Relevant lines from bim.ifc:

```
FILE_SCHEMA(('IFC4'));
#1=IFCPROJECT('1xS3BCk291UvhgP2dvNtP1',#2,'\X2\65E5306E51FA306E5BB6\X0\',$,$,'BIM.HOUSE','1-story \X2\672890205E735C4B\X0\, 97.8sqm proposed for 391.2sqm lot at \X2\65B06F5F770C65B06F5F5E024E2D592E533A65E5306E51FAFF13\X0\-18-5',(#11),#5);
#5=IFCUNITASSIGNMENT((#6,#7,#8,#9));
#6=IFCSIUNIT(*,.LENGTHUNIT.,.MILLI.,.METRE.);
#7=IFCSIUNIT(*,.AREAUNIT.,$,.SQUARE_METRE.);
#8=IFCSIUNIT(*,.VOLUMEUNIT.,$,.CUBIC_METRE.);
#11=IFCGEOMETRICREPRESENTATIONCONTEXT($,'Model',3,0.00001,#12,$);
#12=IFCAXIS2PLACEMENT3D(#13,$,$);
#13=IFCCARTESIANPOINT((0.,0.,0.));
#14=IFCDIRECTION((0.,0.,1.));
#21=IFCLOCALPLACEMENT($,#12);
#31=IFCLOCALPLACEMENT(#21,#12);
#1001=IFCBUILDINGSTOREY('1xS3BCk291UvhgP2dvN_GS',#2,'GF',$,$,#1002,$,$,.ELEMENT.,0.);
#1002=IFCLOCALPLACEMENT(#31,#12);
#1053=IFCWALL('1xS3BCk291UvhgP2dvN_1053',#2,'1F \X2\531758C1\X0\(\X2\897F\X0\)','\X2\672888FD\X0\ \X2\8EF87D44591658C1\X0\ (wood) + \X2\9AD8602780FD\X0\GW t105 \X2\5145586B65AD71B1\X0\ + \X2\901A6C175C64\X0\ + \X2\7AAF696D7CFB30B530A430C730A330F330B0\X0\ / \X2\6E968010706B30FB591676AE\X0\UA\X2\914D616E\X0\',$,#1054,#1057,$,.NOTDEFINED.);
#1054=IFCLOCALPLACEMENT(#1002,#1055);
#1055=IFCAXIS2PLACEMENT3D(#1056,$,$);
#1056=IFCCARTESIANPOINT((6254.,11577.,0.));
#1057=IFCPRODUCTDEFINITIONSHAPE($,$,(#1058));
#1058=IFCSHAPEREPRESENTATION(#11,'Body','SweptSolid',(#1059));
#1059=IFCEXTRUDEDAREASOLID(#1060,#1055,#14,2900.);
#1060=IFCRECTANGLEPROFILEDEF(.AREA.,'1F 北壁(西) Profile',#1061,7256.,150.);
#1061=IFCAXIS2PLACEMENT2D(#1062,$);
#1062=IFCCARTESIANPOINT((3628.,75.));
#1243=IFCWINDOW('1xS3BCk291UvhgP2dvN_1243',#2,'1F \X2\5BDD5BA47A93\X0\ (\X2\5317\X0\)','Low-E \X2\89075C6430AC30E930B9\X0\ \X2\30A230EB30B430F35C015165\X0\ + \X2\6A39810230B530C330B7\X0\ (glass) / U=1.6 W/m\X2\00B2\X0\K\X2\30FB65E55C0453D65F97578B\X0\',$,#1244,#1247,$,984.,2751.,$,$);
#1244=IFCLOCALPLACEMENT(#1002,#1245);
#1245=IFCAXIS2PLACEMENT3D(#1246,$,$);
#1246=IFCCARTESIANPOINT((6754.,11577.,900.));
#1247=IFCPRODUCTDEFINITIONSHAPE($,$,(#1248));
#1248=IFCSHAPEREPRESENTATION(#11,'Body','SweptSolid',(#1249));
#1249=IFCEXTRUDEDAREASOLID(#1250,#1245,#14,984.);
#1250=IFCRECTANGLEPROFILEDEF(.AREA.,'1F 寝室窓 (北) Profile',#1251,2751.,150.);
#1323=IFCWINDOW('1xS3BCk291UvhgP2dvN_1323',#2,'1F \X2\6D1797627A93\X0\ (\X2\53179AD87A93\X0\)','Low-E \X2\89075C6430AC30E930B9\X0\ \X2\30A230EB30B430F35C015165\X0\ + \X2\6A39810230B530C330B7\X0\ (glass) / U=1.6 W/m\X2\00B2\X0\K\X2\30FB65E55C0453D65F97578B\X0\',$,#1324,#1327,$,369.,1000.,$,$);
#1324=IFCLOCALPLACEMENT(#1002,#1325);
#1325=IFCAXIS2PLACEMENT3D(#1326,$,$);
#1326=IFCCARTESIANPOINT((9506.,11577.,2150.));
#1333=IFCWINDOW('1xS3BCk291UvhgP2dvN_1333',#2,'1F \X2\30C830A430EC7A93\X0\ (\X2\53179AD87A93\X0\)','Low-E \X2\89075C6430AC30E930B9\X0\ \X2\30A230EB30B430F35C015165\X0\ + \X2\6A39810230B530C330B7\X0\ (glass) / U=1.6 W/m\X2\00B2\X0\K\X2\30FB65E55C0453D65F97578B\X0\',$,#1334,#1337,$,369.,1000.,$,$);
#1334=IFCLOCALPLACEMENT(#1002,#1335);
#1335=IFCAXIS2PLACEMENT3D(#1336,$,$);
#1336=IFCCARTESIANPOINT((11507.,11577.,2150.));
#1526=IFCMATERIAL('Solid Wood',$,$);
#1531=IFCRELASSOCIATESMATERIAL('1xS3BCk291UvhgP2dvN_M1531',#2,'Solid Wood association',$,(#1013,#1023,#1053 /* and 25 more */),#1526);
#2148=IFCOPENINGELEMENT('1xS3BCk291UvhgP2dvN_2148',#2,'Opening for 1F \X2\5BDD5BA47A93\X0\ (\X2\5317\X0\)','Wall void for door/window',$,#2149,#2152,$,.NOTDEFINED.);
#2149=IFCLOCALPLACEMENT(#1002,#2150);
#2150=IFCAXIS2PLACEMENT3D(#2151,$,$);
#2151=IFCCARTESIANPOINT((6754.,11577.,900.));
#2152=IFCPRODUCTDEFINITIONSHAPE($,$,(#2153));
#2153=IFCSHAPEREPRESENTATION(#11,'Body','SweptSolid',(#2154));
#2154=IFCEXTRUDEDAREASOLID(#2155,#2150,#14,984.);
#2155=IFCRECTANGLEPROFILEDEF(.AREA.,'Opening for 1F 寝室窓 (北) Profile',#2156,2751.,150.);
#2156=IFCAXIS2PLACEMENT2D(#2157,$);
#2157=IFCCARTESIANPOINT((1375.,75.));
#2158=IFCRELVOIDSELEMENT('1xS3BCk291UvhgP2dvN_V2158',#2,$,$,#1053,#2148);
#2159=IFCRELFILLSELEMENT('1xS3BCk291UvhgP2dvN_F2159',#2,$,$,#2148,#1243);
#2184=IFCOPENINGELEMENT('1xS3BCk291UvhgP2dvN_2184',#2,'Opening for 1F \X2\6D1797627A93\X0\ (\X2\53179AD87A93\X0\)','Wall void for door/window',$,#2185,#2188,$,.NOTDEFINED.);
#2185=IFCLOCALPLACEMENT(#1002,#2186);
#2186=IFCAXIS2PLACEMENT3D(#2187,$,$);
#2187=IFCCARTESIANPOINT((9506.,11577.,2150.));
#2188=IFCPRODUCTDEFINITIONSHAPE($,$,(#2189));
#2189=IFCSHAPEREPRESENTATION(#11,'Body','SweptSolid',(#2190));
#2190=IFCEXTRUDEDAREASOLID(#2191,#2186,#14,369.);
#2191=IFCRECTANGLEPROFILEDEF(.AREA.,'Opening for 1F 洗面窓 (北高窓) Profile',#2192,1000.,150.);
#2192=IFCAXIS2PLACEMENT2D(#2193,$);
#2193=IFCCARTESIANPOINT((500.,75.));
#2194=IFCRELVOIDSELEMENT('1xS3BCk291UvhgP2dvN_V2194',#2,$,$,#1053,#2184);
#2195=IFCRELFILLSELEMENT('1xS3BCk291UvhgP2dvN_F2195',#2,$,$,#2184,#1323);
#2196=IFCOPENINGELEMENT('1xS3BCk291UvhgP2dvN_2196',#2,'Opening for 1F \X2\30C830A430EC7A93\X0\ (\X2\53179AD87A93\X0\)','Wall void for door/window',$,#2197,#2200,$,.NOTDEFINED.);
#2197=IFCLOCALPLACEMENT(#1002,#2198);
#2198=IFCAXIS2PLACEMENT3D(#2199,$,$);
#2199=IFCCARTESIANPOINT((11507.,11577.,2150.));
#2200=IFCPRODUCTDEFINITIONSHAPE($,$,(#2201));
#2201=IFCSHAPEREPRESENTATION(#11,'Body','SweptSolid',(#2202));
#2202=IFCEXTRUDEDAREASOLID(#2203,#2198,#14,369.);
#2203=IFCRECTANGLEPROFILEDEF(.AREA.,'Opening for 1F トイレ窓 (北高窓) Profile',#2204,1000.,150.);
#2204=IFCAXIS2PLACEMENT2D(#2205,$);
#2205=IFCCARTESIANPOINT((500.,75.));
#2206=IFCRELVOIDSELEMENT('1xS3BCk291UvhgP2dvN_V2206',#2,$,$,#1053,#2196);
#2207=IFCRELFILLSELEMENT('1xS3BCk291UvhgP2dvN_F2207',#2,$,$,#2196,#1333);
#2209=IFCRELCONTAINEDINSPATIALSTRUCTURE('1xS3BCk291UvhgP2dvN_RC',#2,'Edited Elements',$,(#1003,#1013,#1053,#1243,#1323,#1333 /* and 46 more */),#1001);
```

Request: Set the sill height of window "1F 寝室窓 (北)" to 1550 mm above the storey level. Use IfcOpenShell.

```python
import numpy as np
import ifcopenshell
import ifcopenshell.api.geometry
import ifcopenshell.geom
import ifcopenshell.util.element
import ifcopenshell.util.placement
import ifcopenshell.util.shape
import ifcopenshell.util.unit

model = ifcopenshell.open("bim.ifc")
unit_scale = ifcopenshell.util.unit.calculate_unit_scale(model)

window = model.by_guid("1xS3BCk291UvhgP2dvN_1243")
opening = window.FillsVoids[0].RelatingOpeningElement
storey = ifcopenshell.util.element.get_container(window, ifc_class="IfcBuildingStorey")
level = ifcopenshell.util.placement.get_local_placement(storey.ObjectPlacement)[2, 3]

# The opening's origin need not be at the sill, so measure its lowest point.
shape = ifcopenshell.geom.create_shape(ifcopenshell.geom.settings(), opening)
bottom = ifcopenshell.util.shape.get_shape_bottom_elevation(shape, shape.geometry) / unit_scale
dz = level + 1.55 / unit_scale - bottom

shift = np.array([0.0, 0.0, dz])
# The window is not placed relative to its opening, so move both.
for product in (opening, window):
    matrix = ifcopenshell.util.placement.get_local_placement(product.ObjectPlacement)
    matrix[:3, 3] += shift
    ifcopenshell.api.geometry.edit_object_placement(model, product=product, matrix=matrix, is_si=False)

print(f"moved by {dz * unit_scale:+.3f} m")

model.write("bim_edited.ifc")
```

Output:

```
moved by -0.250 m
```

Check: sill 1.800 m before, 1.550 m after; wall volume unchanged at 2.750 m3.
